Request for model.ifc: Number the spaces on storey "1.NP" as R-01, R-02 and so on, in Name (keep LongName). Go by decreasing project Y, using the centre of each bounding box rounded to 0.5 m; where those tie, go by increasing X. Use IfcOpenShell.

First a look at what the model holds.

```python
import ifcopenshell
import ifcopenshell.util.element
import ifcopenshell.util.placement

model = ifcopenshell.open("model.ifc")
print(model.schema)
storey = next(s for s in model.by_type("IfcBuildingStorey") if s.Name == "1.NP")
spaces = [e for e in ifcopenshell.util.element.get_decomposition(storey) if e.is_a("IfcSpace")]
for e in sorted(spaces, key=lambda e: e.id()):
    origin = ifcopenshell.util.placement.get_local_placement(e.ObjectPlacement)[:3, 3]
    print(e.id(), e.Name, e.LongName, origin.round(2) + 0.0, sep=" | ")
```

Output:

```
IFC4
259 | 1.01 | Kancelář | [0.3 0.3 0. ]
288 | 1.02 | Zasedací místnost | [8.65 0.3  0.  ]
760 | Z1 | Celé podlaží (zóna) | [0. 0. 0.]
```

```python
import ifcopenshell
import ifcopenshell.geom
import ifcopenshell.util.element
import ifcopenshell.util.shape

model = ifcopenshell.open("model.ifc")
settings = ifcopenshell.geom.settings()
settings.set("use-world-coords", True)


def centre(element):
    shape = ifcopenshell.geom.create_shape(settings, element)
    return ifcopenshell.util.shape.get_bbox_centroid(shape.geometry)


storey = next(s for s in model.by_type("IfcBuildingStorey") if s.Name == "1.NP")
spaces = [e for e in ifcopenshell.util.element.get_decomposition(storey) if e.is_a("IfcSpace")]

# Insertion points can sit at a corner or the storey origin, so sort by the geometry (in metres).
centres = {e: centre(e) for e in spaces}
spaces.sort(key=lambda e: (-round(centres[e][1] / 0.5), centres[e][0]))

for i, e in enumerate(spaces, start=1):
    number = f"R-{i:02d}"
    e.Name = number
    print(e.id(), number)

model.write("model_edited.ifc")
```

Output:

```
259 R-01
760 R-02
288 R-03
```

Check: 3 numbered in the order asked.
